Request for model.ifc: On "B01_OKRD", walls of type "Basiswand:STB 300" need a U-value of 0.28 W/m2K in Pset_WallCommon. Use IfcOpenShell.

First a look at what the model holds.

```python
import ifcopenshell
import ifcopenshell.util.element

model = ifcopenshell.open("model.ifc")
print(model.schema)
storey = next(s for s in model.by_type("IfcBuildingStorey") if s.Name == "B01_OKRD")
walls = [e for e in ifcopenshell.util.element.get_decomposition(storey) if e.is_a("IfcWall")]
seen = {}
for e in walls:
    element_type = ifcopenshell.util.element.get_type(e)
    key = (element_type.Name if element_type != e and element_type else None, ifcopenshell.util.element.get_pset(e, "Pset_WallCommon", "ThermalTransmittance"))
    seen[key] = seen.get(key, 0) + 1
for (name, value), count in sorted(seen.items(), key=str):
    print(count, "x", name, "|", value)
```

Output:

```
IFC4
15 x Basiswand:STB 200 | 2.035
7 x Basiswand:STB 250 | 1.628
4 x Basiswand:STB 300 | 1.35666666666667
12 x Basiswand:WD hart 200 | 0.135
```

```python
import ifcopenshell
import ifcopenshell.api.pset
import ifcopenshell.util.element

model = ifcopenshell.open("model.ifc")

storey = next(s for s in model.by_type("IfcBuildingStorey") if s.Name == "B01_OKRD")
walls = [e for e in ifcopenshell.util.element.get_decomposition(storey) if e.is_a("IfcWall")]

count = 0
for e in walls:
    element_type = ifcopenshell.util.element.get_type(e)
    if element_type in (None, e) or element_type.Name != "Basiswand:STB 300":
        continue
    # add_pset returns the element's existing set when there is one.
    pset = ifcopenshell.api.pset.add_pset(model, product=e, name="Pset_WallCommon")
    ifcopenshell.api.pset.edit_pset(model, pset=pset, properties={"ThermalTransmittance": 0.28})
    count += 1

print(count, "walls updated")

model.write("model-out.ifc")
```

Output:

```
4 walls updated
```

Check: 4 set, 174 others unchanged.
